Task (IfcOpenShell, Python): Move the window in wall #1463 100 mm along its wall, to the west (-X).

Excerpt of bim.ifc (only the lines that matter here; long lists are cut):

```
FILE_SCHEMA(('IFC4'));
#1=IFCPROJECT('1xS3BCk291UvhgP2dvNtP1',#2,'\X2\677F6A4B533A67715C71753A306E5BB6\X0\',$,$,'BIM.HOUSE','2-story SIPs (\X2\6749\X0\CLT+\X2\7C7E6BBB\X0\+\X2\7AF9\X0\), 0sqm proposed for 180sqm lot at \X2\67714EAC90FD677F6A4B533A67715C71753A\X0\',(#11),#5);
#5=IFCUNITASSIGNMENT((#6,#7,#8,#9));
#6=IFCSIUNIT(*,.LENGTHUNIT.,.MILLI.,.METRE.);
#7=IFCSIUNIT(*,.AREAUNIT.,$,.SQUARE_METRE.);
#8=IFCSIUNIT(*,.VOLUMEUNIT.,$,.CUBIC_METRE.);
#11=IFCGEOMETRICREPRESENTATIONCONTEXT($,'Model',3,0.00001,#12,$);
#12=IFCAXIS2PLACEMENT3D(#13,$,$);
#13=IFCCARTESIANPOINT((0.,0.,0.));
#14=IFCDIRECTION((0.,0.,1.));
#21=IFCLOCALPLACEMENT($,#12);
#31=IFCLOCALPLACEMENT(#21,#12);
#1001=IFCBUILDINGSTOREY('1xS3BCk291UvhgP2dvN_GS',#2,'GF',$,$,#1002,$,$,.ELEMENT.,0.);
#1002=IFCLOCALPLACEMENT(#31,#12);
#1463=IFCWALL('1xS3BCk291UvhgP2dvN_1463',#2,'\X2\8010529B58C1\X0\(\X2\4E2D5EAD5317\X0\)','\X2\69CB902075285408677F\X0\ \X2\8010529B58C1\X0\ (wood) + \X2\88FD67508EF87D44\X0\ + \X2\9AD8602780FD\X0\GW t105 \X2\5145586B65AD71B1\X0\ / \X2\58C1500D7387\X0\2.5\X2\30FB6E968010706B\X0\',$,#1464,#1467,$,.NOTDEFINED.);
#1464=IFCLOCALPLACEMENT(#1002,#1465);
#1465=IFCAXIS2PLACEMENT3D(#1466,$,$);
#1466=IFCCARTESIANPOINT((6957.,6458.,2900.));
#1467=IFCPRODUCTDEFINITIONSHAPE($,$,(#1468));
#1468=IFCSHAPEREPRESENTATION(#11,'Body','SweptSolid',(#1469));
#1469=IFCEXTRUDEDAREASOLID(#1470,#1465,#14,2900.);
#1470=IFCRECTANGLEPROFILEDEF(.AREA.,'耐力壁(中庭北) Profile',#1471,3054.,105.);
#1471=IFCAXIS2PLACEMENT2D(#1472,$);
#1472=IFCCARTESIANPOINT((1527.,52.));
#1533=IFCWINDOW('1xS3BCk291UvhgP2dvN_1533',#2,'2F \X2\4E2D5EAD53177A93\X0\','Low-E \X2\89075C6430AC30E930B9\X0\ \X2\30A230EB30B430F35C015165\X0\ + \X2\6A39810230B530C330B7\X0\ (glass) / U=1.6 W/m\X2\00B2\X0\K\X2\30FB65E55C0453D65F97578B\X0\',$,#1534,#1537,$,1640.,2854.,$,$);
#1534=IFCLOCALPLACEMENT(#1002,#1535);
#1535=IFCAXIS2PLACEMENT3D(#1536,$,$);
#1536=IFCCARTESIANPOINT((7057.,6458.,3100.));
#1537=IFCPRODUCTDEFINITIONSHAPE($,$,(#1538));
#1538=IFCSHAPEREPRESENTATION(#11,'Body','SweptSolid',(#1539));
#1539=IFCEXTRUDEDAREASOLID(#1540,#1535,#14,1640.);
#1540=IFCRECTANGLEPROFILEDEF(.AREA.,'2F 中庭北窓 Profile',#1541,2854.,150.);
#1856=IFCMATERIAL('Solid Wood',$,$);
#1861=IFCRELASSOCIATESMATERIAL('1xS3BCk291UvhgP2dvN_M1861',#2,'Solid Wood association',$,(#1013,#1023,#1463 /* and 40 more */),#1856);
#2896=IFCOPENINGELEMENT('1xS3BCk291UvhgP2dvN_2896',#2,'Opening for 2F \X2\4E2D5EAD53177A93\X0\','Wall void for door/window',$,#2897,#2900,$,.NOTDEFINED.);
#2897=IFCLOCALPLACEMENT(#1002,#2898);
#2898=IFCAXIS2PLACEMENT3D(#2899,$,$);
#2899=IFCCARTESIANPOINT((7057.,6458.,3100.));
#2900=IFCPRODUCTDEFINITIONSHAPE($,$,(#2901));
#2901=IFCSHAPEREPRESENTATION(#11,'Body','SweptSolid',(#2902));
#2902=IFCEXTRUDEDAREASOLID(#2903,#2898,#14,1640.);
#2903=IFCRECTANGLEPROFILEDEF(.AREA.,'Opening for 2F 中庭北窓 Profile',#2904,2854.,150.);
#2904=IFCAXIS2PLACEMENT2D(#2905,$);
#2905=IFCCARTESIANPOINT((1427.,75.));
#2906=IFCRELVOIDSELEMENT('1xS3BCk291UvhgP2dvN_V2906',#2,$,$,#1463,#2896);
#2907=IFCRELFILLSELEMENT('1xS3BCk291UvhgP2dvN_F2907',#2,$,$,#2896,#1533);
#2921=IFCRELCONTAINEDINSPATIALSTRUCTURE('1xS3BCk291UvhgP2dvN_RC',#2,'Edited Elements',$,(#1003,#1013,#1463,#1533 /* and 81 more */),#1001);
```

```python
import ifcopenshell
import ifcopenshell.api.geometry
import ifcopenshell.util.placement
import ifcopenshell.util.unit

model = ifcopenshell.open("bim.ifc")
unit_scale = ifcopenshell.util.unit.calculate_unit_scale(model)

window = model.by_guid("1xS3BCk291UvhgP2dvN_1533")
opening = window.FillsVoids[0].RelatingOpeningElement
wall = opening.VoidsElements[0].RelatingBuildingElement

wall_matrix = ifcopenshell.util.placement.get_local_placement(wall.ObjectPlacement)
shift = wall_matrix[:3, 0] * -0.1 / unit_scale
before = ifcopenshell.util.placement.get_local_placement(window.ObjectPlacement)[:3, 3].copy()

# The window is not placed relative to its opening, so move both.
for product in (opening, window):
    matrix = ifcopenshell.util.placement.get_local_placement(product.ObjectPlacement)
    matrix[:3, 3] += shift
    ifcopenshell.api.geometry.edit_object_placement(model, product=product, matrix=matrix, is_si=False)

after = ifcopenshell.util.placement.get_local_placement(window.ObjectPlacement)[:3, 3]
print("window moved by", (after - before).round(3) + 0.0)

model.write("bim_v2.ifc")
```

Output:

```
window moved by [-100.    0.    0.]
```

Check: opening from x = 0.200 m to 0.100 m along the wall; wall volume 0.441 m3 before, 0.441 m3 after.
